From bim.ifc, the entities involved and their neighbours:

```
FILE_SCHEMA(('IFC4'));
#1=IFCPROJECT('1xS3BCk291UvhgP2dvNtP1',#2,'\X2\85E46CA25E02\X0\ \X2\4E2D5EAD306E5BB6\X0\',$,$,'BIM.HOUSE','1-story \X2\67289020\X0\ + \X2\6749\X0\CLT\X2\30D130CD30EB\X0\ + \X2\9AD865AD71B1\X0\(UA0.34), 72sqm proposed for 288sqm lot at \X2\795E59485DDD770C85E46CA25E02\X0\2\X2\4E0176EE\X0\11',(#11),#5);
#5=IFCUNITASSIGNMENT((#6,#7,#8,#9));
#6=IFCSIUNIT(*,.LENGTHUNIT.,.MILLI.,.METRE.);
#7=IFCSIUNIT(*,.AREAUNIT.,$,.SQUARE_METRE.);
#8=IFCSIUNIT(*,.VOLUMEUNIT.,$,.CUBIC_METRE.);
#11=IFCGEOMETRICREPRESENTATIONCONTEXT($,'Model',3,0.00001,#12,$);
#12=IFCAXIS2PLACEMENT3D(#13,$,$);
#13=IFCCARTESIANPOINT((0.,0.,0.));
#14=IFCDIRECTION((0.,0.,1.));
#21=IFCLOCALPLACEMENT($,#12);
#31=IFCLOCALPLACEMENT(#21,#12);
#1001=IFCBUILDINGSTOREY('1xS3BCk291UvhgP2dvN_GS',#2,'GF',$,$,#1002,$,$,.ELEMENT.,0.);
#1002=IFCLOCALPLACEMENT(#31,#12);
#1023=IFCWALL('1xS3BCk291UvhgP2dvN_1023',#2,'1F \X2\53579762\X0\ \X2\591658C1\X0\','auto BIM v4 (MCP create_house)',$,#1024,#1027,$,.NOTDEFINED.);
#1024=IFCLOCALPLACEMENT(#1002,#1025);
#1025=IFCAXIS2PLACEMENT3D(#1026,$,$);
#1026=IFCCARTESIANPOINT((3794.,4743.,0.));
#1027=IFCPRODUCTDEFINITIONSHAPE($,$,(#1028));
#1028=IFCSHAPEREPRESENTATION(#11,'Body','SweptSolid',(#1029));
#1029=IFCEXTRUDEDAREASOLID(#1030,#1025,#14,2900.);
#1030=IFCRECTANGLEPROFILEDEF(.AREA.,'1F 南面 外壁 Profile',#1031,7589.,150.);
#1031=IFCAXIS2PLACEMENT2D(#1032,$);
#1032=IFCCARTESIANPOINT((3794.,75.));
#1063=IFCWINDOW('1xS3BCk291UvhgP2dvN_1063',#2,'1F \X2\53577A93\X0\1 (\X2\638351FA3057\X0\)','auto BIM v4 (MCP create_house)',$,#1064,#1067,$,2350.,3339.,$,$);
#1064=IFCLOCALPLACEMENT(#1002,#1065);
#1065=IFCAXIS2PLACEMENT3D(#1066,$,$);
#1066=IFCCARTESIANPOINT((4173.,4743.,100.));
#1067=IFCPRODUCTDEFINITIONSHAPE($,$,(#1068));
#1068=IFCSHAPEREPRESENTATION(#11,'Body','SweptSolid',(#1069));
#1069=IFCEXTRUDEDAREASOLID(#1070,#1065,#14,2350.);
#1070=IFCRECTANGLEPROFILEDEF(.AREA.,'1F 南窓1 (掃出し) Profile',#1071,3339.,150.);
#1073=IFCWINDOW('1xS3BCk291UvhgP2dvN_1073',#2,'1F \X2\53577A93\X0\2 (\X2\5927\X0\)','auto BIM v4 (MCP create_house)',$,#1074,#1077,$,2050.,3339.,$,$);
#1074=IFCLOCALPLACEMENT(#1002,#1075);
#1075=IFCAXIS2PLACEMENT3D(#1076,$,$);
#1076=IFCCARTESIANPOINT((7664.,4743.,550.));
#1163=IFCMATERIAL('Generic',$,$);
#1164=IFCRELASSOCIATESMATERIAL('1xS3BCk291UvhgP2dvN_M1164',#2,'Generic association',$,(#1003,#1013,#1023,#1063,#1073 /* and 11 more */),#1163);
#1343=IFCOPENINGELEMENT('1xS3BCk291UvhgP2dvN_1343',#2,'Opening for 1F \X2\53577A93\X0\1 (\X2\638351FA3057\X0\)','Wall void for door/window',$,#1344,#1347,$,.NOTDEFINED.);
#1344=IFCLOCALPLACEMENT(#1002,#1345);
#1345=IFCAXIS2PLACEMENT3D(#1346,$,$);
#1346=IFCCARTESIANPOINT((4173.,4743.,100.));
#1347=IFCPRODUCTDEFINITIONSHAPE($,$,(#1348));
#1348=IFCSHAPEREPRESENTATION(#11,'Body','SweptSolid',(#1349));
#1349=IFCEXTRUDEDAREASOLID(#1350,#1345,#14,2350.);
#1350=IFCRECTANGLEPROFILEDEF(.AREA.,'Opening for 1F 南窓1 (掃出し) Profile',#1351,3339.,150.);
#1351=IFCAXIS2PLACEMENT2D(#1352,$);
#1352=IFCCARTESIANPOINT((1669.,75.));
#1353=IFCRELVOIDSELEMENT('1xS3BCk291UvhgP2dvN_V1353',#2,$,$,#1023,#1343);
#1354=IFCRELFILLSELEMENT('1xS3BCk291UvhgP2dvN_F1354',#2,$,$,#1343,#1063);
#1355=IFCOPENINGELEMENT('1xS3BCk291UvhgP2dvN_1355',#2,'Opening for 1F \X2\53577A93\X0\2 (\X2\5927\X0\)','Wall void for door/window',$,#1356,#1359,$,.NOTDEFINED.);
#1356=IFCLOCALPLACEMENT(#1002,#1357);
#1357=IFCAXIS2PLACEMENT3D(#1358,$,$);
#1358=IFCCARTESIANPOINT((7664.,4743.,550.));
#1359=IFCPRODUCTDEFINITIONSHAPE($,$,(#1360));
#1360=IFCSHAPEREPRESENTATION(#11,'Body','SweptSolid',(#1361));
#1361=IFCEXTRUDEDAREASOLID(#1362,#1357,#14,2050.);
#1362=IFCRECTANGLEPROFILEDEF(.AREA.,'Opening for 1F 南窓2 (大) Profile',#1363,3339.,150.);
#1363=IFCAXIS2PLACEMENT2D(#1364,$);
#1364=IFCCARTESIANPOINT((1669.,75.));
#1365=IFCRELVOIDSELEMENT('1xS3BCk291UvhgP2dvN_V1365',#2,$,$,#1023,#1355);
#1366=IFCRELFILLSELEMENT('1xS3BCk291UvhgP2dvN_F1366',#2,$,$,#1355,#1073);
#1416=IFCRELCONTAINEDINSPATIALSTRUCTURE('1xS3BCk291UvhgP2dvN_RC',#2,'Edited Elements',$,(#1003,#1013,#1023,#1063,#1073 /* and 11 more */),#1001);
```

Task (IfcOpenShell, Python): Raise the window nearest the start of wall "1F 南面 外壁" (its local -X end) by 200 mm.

```python
import numpy as np
import ifcopenshell
import ifcopenshell.api.geometry
import ifcopenshell.util.placement
import ifcopenshell.util.unit

model = ifcopenshell.open("bim.ifc")
unit_scale = ifcopenshell.util.unit.calculate_unit_scale(model)

window = model.by_id(1063)
opening = window.FillsVoids[0].RelatingOpeningElement
dz = 200.0

shift = np.array([0.0, 0.0, dz])
# The window is not placed relative to its opening, so move both.
for product in (opening, window):
    matrix = ifcopenshell.util.placement.get_local_placement(product.ObjectPlacement)
    matrix[:3, 3] += shift
    ifcopenshell.api.geometry.edit_object_placement(model, product=product, matrix=matrix, is_si=False)

print(f"moved by {dz * unit_scale:+.3f} m")

model.write("bim_rev.ifc")
```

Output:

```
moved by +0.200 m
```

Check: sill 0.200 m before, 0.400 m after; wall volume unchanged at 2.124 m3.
